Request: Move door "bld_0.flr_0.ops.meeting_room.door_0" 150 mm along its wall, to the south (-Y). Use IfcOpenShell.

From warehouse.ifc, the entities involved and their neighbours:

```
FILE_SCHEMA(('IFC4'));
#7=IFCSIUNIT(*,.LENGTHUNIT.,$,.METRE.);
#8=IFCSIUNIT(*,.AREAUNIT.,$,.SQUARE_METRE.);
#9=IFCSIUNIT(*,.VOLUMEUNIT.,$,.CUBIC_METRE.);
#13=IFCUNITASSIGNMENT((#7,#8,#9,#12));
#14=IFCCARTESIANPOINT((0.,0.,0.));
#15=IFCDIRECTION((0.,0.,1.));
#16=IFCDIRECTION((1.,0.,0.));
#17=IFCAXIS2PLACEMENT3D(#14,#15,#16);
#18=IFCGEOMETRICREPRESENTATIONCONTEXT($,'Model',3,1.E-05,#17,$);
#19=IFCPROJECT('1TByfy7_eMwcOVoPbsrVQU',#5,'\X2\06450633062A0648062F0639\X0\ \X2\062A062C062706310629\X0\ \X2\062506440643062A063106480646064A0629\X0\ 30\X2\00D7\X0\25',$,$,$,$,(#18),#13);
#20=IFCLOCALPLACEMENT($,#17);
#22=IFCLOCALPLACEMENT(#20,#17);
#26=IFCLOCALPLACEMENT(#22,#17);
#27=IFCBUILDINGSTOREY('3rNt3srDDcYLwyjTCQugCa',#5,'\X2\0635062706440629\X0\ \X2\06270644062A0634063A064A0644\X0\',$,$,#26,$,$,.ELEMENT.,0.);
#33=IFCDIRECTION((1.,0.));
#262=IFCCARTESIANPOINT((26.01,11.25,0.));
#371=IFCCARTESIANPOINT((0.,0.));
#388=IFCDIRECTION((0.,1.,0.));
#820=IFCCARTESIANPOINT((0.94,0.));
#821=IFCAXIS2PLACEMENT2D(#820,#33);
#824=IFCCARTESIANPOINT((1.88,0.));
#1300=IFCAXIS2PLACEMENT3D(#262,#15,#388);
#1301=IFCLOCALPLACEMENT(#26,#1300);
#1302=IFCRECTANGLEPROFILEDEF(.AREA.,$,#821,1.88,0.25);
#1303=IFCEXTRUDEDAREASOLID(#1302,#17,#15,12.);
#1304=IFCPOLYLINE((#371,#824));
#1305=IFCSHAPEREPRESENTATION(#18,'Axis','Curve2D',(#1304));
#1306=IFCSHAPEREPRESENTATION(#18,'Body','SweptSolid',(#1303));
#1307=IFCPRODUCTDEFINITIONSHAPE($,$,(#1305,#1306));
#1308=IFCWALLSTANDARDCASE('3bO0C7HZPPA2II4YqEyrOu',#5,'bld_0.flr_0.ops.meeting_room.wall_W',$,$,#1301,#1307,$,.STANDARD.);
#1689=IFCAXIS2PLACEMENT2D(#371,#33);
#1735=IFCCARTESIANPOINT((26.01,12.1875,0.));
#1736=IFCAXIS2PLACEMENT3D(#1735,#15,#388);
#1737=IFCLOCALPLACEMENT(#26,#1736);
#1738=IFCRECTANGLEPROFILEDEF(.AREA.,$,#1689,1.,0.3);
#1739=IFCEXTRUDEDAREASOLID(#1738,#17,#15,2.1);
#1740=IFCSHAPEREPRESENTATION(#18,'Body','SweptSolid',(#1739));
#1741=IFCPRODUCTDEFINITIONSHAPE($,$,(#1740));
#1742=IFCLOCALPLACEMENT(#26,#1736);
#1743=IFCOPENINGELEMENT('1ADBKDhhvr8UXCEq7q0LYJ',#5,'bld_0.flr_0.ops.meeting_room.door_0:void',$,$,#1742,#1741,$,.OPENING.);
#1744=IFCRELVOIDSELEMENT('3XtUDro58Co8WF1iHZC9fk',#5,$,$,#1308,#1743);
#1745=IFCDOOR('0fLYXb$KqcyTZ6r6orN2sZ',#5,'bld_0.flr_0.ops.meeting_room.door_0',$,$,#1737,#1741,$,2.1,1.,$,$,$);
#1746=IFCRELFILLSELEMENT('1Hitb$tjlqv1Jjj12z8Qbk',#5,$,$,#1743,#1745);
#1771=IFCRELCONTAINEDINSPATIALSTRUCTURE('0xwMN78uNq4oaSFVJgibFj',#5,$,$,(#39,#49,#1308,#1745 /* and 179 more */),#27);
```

```python
import ifcopenshell
import ifcopenshell.api.geometry
import ifcopenshell.util.placement

model = ifcopenshell.open("warehouse.ifc")

door = model.by_guid("0fLYXb$KqcyTZ6r6orN2sZ")
opening = door.FillsVoids[0].RelatingOpeningElement
wall = opening.VoidsElements[0].RelatingBuildingElement

wall_matrix = ifcopenshell.util.placement.get_local_placement(wall.ObjectPlacement)
shift = wall_matrix[:3, 0] * -0.15
before = ifcopenshell.util.placement.get_local_placement(door.ObjectPlacement)[:3, 3].copy()

# The door is not placed relative to its opening, so move both.
for product in (opening, door):
    matrix = ifcopenshell.util.placement.get_local_placement(product.ObjectPlacement)
    matrix[:3, 3] += shift
    ifcopenshell.api.geometry.edit_object_placement(model, product=product, matrix=matrix, is_si=False)

after = ifcopenshell.util.placement.get_local_placement(door.ObjectPlacement)[:3, 3]
print("door moved by", (after - before).round(3) + 0.0)

model.write("warehouse_rev.ifc")
```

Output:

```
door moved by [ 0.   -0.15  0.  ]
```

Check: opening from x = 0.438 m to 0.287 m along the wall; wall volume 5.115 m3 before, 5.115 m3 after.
